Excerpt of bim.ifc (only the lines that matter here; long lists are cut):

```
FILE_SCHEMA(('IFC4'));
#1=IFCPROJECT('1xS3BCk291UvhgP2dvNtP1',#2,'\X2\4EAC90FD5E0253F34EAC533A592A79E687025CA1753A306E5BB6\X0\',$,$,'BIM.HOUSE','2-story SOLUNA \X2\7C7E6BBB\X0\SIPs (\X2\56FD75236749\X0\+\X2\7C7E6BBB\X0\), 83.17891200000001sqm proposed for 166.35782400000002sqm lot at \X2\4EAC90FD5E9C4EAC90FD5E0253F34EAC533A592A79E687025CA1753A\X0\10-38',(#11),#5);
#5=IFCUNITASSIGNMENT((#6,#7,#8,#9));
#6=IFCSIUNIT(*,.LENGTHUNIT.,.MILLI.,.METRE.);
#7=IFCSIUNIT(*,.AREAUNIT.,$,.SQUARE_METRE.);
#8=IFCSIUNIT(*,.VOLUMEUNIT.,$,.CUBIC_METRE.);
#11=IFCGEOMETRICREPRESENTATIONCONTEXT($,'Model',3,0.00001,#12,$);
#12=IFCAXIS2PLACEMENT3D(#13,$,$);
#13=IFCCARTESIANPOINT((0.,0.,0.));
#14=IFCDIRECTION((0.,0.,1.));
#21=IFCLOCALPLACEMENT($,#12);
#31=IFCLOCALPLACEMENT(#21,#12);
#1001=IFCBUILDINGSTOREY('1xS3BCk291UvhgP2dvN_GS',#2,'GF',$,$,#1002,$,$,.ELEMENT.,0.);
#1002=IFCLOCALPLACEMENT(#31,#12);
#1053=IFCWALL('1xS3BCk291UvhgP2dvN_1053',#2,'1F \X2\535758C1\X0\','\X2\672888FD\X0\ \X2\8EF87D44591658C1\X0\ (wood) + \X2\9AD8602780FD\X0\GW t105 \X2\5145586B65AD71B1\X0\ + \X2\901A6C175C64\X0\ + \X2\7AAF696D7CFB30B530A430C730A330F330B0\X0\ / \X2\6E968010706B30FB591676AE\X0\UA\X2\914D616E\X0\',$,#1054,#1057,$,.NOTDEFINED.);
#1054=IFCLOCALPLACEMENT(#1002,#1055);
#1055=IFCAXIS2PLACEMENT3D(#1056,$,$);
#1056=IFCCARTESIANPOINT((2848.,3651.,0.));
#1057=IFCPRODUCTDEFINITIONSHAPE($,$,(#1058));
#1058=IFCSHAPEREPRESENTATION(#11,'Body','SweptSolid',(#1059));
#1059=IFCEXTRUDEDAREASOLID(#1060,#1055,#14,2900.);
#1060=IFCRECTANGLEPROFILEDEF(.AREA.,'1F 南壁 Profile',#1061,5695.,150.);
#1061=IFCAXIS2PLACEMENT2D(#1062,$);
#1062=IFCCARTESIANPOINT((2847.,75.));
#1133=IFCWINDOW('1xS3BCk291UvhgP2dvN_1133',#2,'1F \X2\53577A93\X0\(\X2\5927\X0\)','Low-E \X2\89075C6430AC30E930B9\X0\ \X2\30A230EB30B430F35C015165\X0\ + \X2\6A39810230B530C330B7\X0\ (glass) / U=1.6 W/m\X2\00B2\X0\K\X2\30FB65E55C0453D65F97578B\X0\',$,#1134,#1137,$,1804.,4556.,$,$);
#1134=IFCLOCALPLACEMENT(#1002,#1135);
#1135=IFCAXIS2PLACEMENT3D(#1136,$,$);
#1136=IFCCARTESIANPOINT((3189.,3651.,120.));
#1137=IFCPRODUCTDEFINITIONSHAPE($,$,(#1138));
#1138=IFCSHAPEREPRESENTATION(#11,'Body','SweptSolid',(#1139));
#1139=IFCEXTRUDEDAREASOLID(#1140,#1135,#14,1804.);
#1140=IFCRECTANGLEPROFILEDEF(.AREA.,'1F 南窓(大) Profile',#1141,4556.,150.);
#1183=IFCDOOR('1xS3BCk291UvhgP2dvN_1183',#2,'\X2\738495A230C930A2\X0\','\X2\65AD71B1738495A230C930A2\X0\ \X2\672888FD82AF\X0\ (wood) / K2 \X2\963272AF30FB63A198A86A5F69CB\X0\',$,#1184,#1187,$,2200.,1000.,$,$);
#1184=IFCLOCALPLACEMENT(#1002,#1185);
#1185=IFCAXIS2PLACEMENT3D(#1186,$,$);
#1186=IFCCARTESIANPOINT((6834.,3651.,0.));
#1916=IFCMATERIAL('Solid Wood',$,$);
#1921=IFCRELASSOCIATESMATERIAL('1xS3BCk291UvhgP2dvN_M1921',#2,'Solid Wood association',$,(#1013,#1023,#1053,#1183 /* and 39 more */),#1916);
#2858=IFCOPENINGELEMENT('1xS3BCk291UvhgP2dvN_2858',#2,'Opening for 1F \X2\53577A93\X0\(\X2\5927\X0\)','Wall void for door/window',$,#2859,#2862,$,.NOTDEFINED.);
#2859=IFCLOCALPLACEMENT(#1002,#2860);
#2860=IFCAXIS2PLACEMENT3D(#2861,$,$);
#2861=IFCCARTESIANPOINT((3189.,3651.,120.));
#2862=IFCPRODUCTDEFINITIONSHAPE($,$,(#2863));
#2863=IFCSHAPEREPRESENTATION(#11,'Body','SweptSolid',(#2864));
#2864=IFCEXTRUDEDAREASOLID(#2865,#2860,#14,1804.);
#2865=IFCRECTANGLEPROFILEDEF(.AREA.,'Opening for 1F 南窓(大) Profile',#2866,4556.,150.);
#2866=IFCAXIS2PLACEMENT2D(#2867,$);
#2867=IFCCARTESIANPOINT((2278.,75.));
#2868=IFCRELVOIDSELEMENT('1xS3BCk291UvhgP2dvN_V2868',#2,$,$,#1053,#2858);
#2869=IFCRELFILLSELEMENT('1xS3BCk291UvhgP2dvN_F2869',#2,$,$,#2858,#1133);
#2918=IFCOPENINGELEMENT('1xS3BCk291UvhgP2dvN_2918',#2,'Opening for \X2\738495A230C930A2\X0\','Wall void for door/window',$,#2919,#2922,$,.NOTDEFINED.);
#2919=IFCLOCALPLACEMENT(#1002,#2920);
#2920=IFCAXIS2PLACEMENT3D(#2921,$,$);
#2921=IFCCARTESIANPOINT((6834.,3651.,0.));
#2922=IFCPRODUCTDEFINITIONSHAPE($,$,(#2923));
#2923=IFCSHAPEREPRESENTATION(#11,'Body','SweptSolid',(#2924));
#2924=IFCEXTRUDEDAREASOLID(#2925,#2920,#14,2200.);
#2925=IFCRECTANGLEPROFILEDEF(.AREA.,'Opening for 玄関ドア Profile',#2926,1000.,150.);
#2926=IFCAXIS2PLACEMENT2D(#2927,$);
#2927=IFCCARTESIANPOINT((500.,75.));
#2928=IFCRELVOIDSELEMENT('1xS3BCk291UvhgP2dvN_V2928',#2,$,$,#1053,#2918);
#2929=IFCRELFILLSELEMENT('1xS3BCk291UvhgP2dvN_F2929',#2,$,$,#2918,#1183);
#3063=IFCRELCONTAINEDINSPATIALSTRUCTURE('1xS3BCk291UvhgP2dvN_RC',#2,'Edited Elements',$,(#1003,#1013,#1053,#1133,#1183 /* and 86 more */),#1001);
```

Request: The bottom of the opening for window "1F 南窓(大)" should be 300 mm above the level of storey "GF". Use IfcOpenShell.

```python
import numpy as np
import ifcopenshell
import ifcopenshell.api.geometry
import ifcopenshell.geom
import ifcopenshell.util.element
import ifcopenshell.util.placement
import ifcopenshell.util.shape
import ifcopenshell.util.unit

model = ifcopenshell.open("bim.ifc")
unit_scale = ifcopenshell.util.unit.calculate_unit_scale(model)

window = model.by_guid("1xS3BCk291UvhgP2dvN_1133")
opening = window.FillsVoids[0].RelatingOpeningElement
storey = ifcopenshell.util.element.get_container(window, ifc_class="IfcBuildingStorey")
level = ifcopenshell.util.placement.get_local_placement(storey.ObjectPlacement)[2, 3]

# The opening's origin need not be at the sill, so measure its lowest point.
shape = ifcopenshell.geom.create_shape(ifcopenshell.geom.settings(), opening)
bottom = ifcopenshell.util.shape.get_shape_bottom_elevation(shape, shape.geometry) / unit_scale
dz = level + 300.0 - bottom

shift = np.array([0.0, 0.0, dz])
# The window is not placed relative to its opening, so move both.
for product in (opening, window):
    matrix = ifcopenshell.util.placement.get_local_placement(product.ObjectPlacement)
    matrix[:3, 3] += shift
    ifcopenshell.api.geometry.edit_object_placement(model, product=product, matrix=matrix, is_si=False)

print(f"moved by {dz * unit_scale:+.3f} m")

model.write("bim-out.ifc")
```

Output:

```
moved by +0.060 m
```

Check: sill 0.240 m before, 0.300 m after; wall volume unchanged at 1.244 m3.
